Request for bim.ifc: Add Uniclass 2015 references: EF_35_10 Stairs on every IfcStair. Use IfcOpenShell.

First a look at what the model holds.

```python
import ifcopenshell

model = ifcopenshell.open("bim.ifc")
print(model.schema)
print("classifications:", [c.Name for c in model.by_type("IfcClassification")])
for ifc_class in ("IfcDoor", "IfcRoof", "IfcStair", "IfcWall", "IfcWindow"):
    print(ifc_class, len(model.by_type(ifc_class)))
```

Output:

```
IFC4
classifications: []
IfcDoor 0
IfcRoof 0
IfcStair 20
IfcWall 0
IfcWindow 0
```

```python
import ifcopenshell
import ifcopenshell.api.classification

model = ifcopenshell.open("bim.ifc")

system = ifcopenshell.api.classification.add_classification(model, classification="Uniclass 2015")

codes = {
    "IfcStair": ("EF_35_10", "Stairs"),
}
for ifc_class, (code, name) in codes.items():
    products = model.by_type(ifc_class)
    ifcopenshell.api.classification.add_reference(
        model, products=products, classification=system, identification=code, name=name
    )
    print(code, len(products))

model.write("bim_v2.ifc")
```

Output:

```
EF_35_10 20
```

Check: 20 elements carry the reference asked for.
